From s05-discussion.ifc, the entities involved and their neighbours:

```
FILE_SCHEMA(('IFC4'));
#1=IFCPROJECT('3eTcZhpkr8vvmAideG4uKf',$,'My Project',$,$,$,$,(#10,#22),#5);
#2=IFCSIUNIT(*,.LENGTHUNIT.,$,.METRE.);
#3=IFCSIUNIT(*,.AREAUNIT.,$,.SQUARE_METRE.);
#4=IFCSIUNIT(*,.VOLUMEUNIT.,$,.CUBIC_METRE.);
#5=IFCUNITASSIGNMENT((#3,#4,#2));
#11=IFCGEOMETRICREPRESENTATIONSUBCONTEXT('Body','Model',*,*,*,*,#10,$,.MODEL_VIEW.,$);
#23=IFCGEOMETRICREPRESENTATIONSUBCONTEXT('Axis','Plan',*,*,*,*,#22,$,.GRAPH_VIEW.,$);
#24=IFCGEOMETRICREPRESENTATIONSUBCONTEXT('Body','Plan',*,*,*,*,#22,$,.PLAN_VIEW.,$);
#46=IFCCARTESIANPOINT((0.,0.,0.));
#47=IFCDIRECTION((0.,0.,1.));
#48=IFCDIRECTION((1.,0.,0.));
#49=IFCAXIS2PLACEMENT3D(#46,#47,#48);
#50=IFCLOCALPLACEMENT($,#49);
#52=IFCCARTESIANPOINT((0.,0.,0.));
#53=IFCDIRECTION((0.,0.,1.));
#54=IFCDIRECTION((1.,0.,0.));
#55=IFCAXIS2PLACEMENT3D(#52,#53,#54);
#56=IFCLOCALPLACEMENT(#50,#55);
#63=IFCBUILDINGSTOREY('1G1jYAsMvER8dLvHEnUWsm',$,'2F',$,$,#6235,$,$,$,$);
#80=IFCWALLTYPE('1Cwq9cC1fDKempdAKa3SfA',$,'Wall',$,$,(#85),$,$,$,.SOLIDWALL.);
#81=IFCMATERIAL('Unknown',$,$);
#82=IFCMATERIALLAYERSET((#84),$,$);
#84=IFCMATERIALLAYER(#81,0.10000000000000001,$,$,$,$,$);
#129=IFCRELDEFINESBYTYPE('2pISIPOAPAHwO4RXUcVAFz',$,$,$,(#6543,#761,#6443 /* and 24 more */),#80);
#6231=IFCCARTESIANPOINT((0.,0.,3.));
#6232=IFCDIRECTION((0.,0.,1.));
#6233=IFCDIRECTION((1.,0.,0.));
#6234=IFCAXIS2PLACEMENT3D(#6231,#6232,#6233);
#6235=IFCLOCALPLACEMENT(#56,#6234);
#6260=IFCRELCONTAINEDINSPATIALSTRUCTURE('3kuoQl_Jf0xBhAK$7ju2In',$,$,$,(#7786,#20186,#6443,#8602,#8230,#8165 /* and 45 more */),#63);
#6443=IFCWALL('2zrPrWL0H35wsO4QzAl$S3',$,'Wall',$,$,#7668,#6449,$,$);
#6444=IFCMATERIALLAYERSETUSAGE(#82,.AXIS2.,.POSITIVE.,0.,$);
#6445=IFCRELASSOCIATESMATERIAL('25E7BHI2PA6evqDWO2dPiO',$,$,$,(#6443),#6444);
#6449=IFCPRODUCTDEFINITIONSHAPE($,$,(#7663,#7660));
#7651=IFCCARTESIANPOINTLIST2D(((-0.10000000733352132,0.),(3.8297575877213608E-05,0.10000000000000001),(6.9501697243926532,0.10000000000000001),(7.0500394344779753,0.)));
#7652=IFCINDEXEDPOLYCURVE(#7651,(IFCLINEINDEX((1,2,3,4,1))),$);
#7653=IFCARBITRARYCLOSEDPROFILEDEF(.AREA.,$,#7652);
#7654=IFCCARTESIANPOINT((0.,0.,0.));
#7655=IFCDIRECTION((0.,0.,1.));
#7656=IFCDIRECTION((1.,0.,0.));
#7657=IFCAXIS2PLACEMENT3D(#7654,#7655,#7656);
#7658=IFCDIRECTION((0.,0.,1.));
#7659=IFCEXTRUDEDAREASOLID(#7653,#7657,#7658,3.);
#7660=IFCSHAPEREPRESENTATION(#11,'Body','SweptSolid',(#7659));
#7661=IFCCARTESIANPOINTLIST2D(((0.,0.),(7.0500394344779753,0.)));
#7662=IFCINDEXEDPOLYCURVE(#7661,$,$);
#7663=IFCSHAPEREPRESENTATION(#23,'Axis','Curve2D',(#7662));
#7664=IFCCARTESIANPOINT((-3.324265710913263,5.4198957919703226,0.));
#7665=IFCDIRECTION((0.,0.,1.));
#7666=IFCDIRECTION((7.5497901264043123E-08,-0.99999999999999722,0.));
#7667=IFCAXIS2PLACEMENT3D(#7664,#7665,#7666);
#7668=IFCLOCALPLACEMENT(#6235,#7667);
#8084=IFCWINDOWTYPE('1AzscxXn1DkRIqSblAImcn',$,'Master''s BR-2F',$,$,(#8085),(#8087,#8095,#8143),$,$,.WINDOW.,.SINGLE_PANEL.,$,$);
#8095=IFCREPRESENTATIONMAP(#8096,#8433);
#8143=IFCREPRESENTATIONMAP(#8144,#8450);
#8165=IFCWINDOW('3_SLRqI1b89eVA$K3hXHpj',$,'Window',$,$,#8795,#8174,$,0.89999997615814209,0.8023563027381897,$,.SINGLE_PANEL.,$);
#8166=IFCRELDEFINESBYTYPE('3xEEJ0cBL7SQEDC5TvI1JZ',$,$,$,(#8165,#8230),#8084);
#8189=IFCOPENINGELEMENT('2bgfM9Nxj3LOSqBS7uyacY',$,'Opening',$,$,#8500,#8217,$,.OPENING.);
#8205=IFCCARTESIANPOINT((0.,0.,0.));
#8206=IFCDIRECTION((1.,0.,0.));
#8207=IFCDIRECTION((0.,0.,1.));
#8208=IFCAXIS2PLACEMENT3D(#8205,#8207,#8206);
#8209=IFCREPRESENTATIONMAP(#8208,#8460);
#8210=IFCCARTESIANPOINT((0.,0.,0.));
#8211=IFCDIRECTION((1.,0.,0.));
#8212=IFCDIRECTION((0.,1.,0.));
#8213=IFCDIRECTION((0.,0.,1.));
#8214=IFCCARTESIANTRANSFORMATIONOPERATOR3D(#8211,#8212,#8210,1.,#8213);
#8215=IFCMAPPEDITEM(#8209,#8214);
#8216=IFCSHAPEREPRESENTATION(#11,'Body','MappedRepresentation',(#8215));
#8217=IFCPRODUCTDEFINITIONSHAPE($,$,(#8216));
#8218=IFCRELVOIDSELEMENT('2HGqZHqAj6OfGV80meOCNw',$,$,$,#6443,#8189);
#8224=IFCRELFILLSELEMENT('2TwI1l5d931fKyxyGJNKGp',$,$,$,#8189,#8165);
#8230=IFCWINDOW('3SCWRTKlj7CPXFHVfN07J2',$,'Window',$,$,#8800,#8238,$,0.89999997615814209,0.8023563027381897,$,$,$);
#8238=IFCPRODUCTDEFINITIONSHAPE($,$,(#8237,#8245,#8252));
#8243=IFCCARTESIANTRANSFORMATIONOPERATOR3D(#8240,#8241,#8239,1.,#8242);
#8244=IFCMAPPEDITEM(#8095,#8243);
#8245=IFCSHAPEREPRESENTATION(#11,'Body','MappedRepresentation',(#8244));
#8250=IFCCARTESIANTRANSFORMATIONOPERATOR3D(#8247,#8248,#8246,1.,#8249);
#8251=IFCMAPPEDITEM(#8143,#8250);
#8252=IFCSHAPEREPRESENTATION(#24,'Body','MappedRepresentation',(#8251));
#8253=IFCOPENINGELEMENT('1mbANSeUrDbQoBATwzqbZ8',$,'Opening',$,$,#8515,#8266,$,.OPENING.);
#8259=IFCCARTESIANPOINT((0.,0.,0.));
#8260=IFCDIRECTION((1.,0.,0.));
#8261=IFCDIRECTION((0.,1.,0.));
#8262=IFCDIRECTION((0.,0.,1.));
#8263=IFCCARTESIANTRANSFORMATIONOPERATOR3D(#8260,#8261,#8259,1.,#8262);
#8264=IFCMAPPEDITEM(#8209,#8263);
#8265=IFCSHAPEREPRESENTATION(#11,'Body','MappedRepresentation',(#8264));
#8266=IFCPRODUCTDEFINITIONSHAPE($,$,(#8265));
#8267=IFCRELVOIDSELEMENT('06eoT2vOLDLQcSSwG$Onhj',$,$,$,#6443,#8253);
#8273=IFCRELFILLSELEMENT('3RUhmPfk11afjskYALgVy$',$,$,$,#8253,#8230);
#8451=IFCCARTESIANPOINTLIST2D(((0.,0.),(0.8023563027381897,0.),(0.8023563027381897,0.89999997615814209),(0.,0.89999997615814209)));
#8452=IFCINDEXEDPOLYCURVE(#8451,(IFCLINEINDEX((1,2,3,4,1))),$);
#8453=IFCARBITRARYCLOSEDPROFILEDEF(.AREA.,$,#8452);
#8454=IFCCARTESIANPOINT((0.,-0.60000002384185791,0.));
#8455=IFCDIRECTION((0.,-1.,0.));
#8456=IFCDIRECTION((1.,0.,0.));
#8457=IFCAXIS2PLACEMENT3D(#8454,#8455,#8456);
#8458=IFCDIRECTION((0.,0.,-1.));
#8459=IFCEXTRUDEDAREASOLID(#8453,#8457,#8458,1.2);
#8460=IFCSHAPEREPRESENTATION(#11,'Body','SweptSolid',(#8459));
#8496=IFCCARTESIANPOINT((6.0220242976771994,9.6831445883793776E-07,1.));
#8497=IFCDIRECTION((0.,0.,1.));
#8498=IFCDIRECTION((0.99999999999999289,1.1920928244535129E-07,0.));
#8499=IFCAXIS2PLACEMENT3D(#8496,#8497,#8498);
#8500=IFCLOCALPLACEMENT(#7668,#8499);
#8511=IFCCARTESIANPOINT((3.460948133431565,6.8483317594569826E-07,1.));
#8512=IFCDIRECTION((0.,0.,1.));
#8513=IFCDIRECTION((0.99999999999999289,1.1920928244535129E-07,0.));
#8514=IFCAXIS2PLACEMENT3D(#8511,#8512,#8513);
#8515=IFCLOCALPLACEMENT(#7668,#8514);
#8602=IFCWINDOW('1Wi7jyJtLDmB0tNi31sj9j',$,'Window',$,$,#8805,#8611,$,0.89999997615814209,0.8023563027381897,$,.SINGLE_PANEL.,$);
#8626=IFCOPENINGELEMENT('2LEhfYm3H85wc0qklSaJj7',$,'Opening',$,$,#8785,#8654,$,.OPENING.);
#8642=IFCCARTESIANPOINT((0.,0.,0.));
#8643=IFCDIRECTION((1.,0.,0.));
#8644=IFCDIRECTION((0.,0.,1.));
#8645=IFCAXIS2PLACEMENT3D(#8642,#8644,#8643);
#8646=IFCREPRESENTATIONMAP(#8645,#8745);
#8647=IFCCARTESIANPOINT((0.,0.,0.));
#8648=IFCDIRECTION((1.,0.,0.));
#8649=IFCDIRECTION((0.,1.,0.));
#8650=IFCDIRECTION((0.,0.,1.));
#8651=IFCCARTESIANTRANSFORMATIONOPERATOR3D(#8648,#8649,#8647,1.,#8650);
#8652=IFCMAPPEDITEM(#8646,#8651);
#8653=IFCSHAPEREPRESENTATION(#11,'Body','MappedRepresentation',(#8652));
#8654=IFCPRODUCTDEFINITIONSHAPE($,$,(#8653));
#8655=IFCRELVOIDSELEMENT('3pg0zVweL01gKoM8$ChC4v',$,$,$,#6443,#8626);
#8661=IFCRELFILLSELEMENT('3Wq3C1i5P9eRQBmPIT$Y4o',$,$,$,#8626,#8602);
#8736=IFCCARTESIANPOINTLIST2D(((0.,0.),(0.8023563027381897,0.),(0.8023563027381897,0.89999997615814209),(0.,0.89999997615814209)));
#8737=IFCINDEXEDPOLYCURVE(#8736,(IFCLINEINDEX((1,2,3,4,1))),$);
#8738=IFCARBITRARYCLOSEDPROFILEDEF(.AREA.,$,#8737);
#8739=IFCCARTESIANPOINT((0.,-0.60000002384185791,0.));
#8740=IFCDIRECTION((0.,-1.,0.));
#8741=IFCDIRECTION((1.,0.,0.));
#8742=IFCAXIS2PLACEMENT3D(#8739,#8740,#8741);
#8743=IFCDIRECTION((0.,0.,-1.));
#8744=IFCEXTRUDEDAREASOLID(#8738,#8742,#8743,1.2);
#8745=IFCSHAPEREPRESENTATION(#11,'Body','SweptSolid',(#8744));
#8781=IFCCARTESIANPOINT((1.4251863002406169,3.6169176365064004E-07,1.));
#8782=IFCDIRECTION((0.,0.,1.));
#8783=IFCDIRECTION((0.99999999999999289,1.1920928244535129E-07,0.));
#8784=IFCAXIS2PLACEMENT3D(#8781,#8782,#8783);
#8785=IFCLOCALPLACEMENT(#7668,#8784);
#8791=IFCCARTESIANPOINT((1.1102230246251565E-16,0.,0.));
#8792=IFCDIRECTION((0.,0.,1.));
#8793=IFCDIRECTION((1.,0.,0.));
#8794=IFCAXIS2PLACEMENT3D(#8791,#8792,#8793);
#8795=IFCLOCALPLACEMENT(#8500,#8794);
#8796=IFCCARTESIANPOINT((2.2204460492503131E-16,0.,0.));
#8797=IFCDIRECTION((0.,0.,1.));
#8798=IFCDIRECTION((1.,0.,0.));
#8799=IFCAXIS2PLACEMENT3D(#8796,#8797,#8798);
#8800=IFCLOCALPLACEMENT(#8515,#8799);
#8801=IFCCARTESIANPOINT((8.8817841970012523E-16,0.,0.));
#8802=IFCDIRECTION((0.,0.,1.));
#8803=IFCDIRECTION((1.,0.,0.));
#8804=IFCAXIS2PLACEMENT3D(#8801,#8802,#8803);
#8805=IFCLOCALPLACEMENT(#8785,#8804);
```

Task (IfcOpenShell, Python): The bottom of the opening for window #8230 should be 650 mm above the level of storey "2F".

```python
import numpy as np
import ifcopenshell
import ifcopenshell.api.geometry
import ifcopenshell.geom
import ifcopenshell.util.element
import ifcopenshell.util.placement
import ifcopenshell.util.shape
import ifcopenshell.util.unit

model = ifcopenshell.open("s05-discussion.ifc")
unit_scale = ifcopenshell.util.unit.calculate_unit_scale(model)

window = model.by_id(8230)
opening = window.FillsVoids[0].RelatingOpeningElement
storey = ifcopenshell.util.element.get_container(window, ifc_class="IfcBuildingStorey")
level = ifcopenshell.util.placement.get_local_placement(storey.ObjectPlacement)[2, 3]

# The opening's origin need not be at the sill, so measure its lowest point.
shape = ifcopenshell.geom.create_shape(ifcopenshell.geom.settings(), opening)
bottom = ifcopenshell.util.shape.get_shape_bottom_elevation(shape, shape.geometry) / unit_scale
dz = level + 0.65 - bottom

shift = np.array([0.0, 0.0, dz])
# The window is placed relative to its opening, so it follows when the opening moves.
matrix = ifcopenshell.util.placement.get_local_placement(opening.ObjectPlacement)
matrix[:3, 3] += shift
ifcopenshell.api.geometry.edit_object_placement(
    model, product=opening, matrix=matrix, is_si=False, should_transform_children=True
)

print(f"moved by {dz * unit_scale:+.3f} m")

model.write("s05-discussion_rev.ifc")
```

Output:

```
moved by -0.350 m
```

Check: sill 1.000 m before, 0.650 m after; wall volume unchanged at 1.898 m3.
